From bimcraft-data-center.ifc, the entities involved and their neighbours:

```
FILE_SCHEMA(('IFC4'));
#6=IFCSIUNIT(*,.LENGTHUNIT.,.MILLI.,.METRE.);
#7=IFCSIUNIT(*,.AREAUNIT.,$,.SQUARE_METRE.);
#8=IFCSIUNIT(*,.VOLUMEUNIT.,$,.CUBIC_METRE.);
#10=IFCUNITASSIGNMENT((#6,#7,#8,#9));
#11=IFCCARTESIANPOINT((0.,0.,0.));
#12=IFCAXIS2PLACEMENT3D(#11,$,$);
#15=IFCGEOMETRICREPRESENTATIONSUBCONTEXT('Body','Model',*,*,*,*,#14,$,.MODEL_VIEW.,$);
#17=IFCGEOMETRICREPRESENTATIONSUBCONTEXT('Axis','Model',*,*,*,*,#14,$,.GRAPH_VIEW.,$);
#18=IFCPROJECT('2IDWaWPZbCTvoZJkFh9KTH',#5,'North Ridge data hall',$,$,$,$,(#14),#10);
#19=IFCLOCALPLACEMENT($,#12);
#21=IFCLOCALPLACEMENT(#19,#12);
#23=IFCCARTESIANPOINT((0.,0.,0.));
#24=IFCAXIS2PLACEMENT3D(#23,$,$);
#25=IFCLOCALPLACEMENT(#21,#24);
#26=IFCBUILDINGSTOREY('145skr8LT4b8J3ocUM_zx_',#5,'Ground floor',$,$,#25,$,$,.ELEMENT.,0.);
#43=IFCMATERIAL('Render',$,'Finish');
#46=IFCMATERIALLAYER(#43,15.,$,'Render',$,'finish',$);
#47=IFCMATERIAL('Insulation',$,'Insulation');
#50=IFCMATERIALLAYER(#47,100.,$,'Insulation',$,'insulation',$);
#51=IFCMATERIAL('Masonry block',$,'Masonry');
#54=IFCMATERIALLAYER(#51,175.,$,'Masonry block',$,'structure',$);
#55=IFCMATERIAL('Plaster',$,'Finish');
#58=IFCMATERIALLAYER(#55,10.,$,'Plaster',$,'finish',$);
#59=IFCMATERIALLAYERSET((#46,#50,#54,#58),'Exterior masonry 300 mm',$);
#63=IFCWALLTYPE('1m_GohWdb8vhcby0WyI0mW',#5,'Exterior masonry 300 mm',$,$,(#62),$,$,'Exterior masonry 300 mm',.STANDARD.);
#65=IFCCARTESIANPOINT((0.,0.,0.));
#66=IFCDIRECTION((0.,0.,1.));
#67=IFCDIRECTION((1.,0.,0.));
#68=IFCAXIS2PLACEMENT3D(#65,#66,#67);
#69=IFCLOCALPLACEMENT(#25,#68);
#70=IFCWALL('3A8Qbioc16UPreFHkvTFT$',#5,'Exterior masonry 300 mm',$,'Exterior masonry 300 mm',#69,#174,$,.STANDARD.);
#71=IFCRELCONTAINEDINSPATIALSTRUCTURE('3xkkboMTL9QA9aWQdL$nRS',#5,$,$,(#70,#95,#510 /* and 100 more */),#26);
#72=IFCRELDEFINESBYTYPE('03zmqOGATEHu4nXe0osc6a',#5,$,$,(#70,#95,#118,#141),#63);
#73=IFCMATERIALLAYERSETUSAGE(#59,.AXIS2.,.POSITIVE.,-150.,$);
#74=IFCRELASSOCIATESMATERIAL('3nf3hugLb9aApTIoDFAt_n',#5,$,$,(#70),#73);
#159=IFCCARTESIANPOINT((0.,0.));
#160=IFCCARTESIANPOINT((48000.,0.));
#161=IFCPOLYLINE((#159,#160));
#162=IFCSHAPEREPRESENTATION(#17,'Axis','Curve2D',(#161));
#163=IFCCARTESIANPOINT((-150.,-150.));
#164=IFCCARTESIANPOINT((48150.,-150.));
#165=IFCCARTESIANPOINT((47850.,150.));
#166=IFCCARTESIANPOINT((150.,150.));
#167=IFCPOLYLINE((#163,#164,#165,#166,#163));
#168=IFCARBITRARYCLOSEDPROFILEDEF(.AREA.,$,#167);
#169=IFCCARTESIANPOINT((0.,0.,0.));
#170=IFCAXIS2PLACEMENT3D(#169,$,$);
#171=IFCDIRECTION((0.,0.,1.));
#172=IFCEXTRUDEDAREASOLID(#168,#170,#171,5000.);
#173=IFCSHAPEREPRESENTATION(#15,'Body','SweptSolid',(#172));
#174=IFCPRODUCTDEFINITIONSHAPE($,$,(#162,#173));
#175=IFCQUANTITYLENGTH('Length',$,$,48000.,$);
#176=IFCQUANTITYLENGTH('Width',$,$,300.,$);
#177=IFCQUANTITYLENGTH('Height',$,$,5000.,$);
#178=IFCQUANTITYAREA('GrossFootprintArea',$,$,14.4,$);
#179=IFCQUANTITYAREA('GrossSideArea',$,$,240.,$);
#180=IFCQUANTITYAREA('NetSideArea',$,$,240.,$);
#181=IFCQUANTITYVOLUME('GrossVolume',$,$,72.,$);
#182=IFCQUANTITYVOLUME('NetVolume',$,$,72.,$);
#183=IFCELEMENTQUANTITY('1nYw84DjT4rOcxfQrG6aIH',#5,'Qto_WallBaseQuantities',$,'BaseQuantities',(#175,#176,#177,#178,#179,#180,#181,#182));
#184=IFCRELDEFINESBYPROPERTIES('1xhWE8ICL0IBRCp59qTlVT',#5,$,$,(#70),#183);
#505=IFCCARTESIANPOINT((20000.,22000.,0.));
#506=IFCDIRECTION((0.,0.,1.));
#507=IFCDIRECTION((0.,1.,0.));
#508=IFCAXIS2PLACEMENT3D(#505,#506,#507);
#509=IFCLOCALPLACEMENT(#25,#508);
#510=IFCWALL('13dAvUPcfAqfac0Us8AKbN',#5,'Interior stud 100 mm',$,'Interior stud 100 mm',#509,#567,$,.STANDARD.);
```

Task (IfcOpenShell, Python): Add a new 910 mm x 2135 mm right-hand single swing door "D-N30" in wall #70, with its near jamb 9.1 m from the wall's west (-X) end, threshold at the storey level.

```python
import numpy as np
import ifcopenshell
import ifcopenshell.api.feature
import ifcopenshell.api.geometry
import ifcopenshell.api.pset
import ifcopenshell.api.root
import ifcopenshell.api.spatial
import ifcopenshell.geom
import ifcopenshell.util.element
import ifcopenshell.util.placement
import ifcopenshell.util.representation
import ifcopenshell.util.shape
import ifcopenshell.util.unit

model = ifcopenshell.open("bimcraft-data-center.ifc")
unit_scale = ifcopenshell.util.unit.calculate_unit_scale(model)
area_scale = ifcopenshell.util.unit.calculate_unit_scale(model, "AREAUNIT")
volume_scale = ifcopenshell.util.unit.calculate_unit_scale(model, "VOLUMEUNIT")
settings = ifcopenshell.geom.settings()


def volume(element):
    """Net volume in cubic metres, openings subtracted."""
    shape = ifcopenshell.geom.create_shape(settings, element)
    return ifcopenshell.util.shape.get_volume(shape.geometry)


wall = model.by_guid("3A8Qbioc16UPreFHkvTFT$")
storey = ifcopenshell.util.element.get_container(wall, ifc_class="IfcBuildingStorey")
context = ifcopenshell.util.representation.get_context(model, "Model", "Body", "MODEL_VIEW")
before = volume(wall)

width, height, from_end, sill = 0.91, 2.135, 9.1, 0.0  # metres

# The wall runs along its own X axis, and the end named is its -X end.
wall_shape = ifcopenshell.geom.create_shape(settings, wall)
x, y, z = ifcopenshell.util.shape.get_vertices(wall_shape.geometry).T
start = x.min() + from_end
face, thickness = float(y.min()), float(y.max() - y.min())
wall_matrix = ifcopenshell.util.placement.get_local_placement(wall.ObjectPlacement)
level = ifcopenshell.util.placement.get_local_placement(storey.ObjectPlacement)[2, 3]


def in_wall(x, y):
    """Placement at x, y metres in the wall's axes, at sill height."""
    matrix = wall_matrix.copy()
    matrix[:, 3] = wall_matrix @ np.array([x / unit_scale, y / unit_scale, 0.0, 1.0])
    matrix[2, 3] = level + sill / unit_scale
    return matrix


# Opening: a box that overshoots both wall faces by 50 mm.
opening = ifcopenshell.api.root.create_entity(model, ifc_class="IfcOpeningElement", predefined_type="OPENING")
box = ifcopenshell.api.geometry.add_wall_representation(
    model, context=context, length=width, height=height, thickness=thickness + 0.1
)
ifcopenshell.api.geometry.assign_representation(model, product=opening, representation=box)
ifcopenshell.api.geometry.edit_object_placement(model, product=opening, matrix=in_wall(start, face - 0.05), is_si=False)
ifcopenshell.api.feature.add_feature(model, feature=opening, element=wall)

door = ifcopenshell.api.root.create_entity(model, ifc_class="IfcDoor", name="D-N30", predefined_type="DOOR")
door.OverallWidth, door.OverallHeight = width / unit_scale, height / unit_scale
door.OperationType = "SINGLE_SWING_RIGHT"
body = ifcopenshell.api.geometry.add_door_representation(
    model,
    context=context,
    overall_width=door.OverallWidth,
    overall_height=door.OverallHeight,
    operation_type="SINGLE_SWING_RIGHT",
    lining_properties={"LiningDepth": thickness / unit_scale, "ThresholdDepth": thickness / unit_scale},
)
ifcopenshell.api.geometry.assign_representation(model, product=door, representation=body)
ifcopenshell.api.spatial.assign_container(model, products=[door], relating_structure=storey)
ifcopenshell.api.feature.add_filling(model, opening=opening, element=door)

# The lining spans the wall, so the door starts at the wall face.
ifcopenshell.api.geometry.edit_object_placement(model, product=door, matrix=in_wall(start, face), is_si=False)

after = volume(wall)

# Update the wall's stored quantities.
qto = model.by_id(ifcopenshell.util.element.get_pset(wall, "Qto_WallBaseQuantities", should_inherit=False)["id"])
ifcopenshell.api.pset.edit_qto(model, qto=qto, properties={
    "NetSideArea": after / thickness / area_scale,
    "NetVolume": after / volume_scale,
})

print(f"wall volume {before:.3f} -> {after:.3f} m3")

model.write("bimcraft-data-center_updated.ifc")
```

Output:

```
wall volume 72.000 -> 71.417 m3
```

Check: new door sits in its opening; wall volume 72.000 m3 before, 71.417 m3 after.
